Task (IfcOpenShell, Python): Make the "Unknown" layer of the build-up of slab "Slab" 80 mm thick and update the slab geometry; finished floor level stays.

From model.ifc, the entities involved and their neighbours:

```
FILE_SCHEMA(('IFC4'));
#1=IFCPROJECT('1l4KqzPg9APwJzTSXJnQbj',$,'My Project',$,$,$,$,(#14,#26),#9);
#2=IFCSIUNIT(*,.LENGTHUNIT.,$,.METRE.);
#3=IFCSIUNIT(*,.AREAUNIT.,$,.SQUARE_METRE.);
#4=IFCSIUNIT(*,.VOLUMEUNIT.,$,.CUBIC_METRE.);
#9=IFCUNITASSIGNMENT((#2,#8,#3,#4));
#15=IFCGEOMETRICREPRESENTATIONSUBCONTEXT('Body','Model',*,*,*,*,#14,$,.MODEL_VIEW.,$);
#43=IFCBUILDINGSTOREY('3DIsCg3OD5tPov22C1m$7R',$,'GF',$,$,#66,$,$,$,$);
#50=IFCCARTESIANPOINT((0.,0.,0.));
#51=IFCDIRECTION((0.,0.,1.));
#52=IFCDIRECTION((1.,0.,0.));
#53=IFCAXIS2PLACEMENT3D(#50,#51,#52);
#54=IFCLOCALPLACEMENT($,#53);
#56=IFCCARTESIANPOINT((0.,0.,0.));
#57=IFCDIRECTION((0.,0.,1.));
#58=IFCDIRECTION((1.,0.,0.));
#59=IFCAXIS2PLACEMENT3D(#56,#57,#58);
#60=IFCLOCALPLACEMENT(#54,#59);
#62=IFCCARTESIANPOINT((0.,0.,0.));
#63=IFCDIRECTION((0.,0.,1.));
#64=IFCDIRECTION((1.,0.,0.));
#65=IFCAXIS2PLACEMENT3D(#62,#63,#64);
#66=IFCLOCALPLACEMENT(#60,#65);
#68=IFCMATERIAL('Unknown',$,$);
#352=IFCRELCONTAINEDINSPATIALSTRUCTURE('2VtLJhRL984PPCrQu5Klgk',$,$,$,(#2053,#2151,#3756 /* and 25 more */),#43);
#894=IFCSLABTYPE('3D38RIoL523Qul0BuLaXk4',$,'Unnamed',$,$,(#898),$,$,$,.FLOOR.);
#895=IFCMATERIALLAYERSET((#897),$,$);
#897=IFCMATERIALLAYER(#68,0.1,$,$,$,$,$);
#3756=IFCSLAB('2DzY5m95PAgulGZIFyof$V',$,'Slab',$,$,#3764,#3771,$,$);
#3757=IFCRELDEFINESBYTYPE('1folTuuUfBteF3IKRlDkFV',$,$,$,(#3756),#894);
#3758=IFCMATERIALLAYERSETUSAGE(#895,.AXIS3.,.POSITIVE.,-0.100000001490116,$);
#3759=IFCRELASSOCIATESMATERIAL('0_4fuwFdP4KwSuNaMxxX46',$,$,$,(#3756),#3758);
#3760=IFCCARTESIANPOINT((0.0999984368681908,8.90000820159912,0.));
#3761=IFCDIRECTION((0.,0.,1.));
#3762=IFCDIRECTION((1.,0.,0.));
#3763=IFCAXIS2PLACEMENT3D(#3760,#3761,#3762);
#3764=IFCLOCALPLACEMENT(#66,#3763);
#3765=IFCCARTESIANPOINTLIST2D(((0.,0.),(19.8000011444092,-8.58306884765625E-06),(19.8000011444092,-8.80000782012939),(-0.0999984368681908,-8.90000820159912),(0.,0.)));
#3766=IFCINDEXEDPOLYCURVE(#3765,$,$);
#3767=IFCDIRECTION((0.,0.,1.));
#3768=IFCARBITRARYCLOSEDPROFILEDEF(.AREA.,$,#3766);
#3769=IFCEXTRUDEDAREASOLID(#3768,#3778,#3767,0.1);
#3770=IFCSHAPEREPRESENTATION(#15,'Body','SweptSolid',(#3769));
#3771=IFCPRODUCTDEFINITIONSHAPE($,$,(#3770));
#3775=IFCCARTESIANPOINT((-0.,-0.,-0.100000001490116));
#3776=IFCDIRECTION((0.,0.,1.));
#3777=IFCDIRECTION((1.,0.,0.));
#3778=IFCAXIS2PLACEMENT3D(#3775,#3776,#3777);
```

```python
import ifcopenshell
import ifcopenshell.util.element
import ifcopenshell.util.representation
import ifcopenshell.util.unit

model = ifcopenshell.open("model.ifc")
unit_scale = ifcopenshell.util.unit.calculate_unit_scale(model)

layer_set = model.by_id(895)
layer = next(l for l in layer_set.MaterialLayers if l.Material and l.Material.Name == "Unknown")
change = 0.08 / unit_scale - layer.LayerThickness
layer.LayerThickness += change

# Geometry does not follow the layer set by itself.
slabs = [e for e in ifcopenshell.util.element.get_elements_by_material(model, layer_set) if e.is_a("IfcSlab")]
for slab in sorted(slabs, key=lambda e: e.id()):
    body = ifcopenshell.util.representation.get_representation(slab, "Model", "Body")
    solid = body.Items[0]
    old_depth = solid.Depth
    solid.Depth += change
    # Extruded upwards: lower the start of the extrusion so the top stays.
    x, y, z = solid.Position.Location.Coordinates
    solid.Position.Location = model.createIfcCartesianPoint((x, y, z - change))
    print(slab.id(), f"{old_depth:g} -> {solid.Depth:g}")

# The layers are counted up from the underside, which has moved.
for usage in {ifcopenshell.util.element.get_material(slab) for slab in slabs}:
    usage.OffsetFromReferenceLine -= change

model.write("model_updated.ifc")
```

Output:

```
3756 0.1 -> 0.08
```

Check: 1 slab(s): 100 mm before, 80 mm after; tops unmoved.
